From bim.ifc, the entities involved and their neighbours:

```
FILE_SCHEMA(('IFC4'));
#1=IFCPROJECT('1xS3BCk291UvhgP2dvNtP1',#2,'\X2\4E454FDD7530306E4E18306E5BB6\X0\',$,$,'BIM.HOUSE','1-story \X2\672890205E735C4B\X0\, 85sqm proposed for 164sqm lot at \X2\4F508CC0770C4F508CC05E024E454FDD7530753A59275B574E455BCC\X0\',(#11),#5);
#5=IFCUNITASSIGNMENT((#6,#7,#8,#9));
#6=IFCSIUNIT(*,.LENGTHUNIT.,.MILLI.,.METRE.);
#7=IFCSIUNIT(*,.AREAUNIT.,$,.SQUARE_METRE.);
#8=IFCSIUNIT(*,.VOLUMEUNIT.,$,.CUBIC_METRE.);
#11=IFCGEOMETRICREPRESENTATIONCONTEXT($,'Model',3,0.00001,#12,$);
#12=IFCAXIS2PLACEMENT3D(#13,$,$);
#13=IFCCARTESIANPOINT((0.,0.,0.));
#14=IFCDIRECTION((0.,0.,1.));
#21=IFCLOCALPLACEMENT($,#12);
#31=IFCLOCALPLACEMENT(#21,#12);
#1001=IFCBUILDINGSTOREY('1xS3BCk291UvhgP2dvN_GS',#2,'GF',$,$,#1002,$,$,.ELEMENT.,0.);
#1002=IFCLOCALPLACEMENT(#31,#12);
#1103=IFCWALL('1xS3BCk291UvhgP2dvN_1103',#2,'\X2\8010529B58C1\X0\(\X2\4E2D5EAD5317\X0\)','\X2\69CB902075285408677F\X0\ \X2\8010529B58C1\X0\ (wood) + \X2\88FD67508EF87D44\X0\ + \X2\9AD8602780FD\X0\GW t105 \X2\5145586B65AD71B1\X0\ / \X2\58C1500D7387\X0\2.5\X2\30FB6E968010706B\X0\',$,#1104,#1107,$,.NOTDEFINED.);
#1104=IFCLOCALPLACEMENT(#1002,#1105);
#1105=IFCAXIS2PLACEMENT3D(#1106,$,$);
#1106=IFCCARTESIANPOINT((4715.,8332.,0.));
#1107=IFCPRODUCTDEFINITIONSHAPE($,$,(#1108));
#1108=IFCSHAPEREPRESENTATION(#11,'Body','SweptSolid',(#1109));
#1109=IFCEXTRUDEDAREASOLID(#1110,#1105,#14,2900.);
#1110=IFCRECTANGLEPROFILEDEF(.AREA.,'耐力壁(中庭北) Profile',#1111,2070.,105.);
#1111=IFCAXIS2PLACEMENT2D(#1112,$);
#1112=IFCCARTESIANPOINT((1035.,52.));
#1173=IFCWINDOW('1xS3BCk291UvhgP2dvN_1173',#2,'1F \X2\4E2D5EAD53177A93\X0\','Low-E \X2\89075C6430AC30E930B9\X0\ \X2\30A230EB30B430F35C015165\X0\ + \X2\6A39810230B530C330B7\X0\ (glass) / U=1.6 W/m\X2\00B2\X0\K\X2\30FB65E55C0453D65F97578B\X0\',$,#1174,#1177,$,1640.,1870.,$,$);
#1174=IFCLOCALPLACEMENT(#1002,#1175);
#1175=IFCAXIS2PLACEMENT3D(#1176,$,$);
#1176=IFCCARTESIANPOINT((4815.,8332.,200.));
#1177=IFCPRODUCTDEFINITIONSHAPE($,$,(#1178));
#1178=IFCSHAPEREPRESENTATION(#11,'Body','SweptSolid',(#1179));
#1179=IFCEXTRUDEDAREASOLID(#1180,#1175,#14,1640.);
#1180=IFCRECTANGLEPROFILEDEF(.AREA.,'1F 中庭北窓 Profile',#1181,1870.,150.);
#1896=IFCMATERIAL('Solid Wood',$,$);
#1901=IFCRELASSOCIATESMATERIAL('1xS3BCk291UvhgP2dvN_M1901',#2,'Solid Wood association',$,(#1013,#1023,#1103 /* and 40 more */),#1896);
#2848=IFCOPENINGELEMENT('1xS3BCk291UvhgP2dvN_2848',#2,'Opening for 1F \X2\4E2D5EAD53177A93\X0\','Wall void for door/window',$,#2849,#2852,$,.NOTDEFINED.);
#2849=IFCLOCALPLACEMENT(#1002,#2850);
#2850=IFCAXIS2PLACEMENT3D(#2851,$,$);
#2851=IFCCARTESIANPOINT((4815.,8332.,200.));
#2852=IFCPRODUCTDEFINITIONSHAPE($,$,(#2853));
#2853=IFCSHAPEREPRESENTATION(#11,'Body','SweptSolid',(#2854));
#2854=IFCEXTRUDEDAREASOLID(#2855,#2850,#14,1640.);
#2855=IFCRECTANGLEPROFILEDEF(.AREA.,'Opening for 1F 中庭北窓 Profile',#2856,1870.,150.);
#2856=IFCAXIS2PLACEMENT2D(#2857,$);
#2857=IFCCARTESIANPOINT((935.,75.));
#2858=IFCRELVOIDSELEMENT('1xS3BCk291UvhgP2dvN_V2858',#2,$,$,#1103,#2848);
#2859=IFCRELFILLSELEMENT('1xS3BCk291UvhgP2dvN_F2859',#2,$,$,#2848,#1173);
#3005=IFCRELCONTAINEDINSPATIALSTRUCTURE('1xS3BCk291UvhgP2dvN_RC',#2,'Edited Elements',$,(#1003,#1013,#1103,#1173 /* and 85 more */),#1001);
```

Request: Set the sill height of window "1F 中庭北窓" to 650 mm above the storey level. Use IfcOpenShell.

```python
import numpy as np
import ifcopenshell
import ifcopenshell.api.geometry
import ifcopenshell.geom
import ifcopenshell.util.element
import ifcopenshell.util.placement
import ifcopenshell.util.shape
import ifcopenshell.util.unit

model = ifcopenshell.open("bim.ifc")
unit_scale = ifcopenshell.util.unit.calculate_unit_scale(model)

window = model.by_guid("1xS3BCk291UvhgP2dvN_1173")
opening = window.FillsVoids[0].RelatingOpeningElement
storey = ifcopenshell.util.element.get_container(window, ifc_class="IfcBuildingStorey")
level = ifcopenshell.util.placement.get_local_placement(storey.ObjectPlacement)[2, 3]

# The opening's origin need not be at the sill, so measure its lowest point.
shape = ifcopenshell.geom.create_shape(ifcopenshell.geom.settings(), opening)
bottom = ifcopenshell.util.shape.get_shape_bottom_elevation(shape, shape.geometry) / unit_scale
dz = level + 0.65 / unit_scale - bottom

shift = np.array([0.0, 0.0, dz])
# The window is not placed relative to its opening, so move both.
for product in (opening, window):
    matrix = ifcopenshell.util.placement.get_local_placement(product.ObjectPlacement)
    matrix[:3, 3] += shift
    ifcopenshell.api.geometry.edit_object_placement(model, product=product, matrix=matrix, is_si=False)

print(f"moved by {dz * unit_scale:+.3f} m")

model.write("bim_v2.ifc")
```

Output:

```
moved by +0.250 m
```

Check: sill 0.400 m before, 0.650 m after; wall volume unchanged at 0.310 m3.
